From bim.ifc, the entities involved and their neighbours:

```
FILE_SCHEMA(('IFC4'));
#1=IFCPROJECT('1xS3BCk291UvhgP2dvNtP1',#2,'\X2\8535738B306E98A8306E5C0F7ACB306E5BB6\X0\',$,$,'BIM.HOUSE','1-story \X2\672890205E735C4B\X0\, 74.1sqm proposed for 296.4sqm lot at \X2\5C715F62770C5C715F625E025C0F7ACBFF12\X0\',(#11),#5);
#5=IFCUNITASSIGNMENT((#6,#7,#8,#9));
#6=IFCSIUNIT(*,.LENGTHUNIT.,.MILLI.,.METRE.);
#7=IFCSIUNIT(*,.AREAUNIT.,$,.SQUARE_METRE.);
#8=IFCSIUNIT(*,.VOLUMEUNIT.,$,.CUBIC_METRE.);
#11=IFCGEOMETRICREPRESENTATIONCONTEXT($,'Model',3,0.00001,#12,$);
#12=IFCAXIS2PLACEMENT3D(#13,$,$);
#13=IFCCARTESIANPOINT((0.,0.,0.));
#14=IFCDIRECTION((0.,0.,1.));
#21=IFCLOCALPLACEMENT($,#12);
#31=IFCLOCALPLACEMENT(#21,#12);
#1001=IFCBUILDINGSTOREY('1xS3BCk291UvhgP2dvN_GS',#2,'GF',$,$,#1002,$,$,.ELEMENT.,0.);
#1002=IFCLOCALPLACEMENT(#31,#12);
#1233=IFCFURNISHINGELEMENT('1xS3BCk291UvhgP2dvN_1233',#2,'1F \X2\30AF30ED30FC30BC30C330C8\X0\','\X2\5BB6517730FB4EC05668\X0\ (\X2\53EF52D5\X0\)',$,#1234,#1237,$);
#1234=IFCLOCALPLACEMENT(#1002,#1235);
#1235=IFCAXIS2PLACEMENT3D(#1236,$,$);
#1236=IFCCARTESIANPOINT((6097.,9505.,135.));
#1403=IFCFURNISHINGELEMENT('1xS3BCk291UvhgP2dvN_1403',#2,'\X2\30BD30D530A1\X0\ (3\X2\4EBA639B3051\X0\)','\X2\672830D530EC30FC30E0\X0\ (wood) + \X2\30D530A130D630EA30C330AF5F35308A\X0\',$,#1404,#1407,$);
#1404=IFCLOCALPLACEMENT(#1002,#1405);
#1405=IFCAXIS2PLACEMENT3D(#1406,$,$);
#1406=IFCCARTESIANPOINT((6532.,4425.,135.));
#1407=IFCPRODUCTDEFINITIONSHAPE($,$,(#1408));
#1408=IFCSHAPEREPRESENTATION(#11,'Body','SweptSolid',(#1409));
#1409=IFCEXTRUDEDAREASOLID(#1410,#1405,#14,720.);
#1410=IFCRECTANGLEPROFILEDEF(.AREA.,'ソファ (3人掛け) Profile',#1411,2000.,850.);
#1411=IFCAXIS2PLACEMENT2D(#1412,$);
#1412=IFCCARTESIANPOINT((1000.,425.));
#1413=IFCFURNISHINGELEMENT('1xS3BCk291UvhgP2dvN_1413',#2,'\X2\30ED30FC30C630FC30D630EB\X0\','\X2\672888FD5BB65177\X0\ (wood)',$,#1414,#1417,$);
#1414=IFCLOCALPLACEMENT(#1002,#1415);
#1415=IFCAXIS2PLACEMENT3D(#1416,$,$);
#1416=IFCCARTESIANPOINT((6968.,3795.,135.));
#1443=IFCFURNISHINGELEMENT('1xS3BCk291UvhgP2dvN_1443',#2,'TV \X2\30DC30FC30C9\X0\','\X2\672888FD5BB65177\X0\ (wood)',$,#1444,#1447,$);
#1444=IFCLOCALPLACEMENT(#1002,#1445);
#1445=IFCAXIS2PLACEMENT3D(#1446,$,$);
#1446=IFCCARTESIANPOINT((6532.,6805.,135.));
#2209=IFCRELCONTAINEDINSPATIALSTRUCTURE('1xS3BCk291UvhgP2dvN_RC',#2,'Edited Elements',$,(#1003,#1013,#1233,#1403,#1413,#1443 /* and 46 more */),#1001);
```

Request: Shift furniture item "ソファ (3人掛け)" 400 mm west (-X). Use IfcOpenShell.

```python
import ifcopenshell
import ifcopenshell.api.geometry
import ifcopenshell.util.placement
import ifcopenshell.util.unit

model = ifcopenshell.open("bim.ifc")
unit_scale = ifcopenshell.util.unit.calculate_unit_scale(model)

item = model.by_guid("1xS3BCk291UvhgP2dvN_1403")
matrix = ifcopenshell.util.placement.get_local_placement(item.ObjectPlacement)
matrix[0, 3] -= 0.4 / unit_scale
ifcopenshell.api.geometry.edit_object_placement(model, product=item, matrix=matrix, is_si=False)

print(ifcopenshell.util.placement.get_local_placement(item.ObjectPlacement).round(3) + 0.0)

model.write("bim-out.ifc")
```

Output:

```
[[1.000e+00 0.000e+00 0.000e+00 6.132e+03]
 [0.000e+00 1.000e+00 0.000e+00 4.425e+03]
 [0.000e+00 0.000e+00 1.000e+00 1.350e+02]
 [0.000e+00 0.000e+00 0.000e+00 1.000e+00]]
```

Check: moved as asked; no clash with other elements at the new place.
